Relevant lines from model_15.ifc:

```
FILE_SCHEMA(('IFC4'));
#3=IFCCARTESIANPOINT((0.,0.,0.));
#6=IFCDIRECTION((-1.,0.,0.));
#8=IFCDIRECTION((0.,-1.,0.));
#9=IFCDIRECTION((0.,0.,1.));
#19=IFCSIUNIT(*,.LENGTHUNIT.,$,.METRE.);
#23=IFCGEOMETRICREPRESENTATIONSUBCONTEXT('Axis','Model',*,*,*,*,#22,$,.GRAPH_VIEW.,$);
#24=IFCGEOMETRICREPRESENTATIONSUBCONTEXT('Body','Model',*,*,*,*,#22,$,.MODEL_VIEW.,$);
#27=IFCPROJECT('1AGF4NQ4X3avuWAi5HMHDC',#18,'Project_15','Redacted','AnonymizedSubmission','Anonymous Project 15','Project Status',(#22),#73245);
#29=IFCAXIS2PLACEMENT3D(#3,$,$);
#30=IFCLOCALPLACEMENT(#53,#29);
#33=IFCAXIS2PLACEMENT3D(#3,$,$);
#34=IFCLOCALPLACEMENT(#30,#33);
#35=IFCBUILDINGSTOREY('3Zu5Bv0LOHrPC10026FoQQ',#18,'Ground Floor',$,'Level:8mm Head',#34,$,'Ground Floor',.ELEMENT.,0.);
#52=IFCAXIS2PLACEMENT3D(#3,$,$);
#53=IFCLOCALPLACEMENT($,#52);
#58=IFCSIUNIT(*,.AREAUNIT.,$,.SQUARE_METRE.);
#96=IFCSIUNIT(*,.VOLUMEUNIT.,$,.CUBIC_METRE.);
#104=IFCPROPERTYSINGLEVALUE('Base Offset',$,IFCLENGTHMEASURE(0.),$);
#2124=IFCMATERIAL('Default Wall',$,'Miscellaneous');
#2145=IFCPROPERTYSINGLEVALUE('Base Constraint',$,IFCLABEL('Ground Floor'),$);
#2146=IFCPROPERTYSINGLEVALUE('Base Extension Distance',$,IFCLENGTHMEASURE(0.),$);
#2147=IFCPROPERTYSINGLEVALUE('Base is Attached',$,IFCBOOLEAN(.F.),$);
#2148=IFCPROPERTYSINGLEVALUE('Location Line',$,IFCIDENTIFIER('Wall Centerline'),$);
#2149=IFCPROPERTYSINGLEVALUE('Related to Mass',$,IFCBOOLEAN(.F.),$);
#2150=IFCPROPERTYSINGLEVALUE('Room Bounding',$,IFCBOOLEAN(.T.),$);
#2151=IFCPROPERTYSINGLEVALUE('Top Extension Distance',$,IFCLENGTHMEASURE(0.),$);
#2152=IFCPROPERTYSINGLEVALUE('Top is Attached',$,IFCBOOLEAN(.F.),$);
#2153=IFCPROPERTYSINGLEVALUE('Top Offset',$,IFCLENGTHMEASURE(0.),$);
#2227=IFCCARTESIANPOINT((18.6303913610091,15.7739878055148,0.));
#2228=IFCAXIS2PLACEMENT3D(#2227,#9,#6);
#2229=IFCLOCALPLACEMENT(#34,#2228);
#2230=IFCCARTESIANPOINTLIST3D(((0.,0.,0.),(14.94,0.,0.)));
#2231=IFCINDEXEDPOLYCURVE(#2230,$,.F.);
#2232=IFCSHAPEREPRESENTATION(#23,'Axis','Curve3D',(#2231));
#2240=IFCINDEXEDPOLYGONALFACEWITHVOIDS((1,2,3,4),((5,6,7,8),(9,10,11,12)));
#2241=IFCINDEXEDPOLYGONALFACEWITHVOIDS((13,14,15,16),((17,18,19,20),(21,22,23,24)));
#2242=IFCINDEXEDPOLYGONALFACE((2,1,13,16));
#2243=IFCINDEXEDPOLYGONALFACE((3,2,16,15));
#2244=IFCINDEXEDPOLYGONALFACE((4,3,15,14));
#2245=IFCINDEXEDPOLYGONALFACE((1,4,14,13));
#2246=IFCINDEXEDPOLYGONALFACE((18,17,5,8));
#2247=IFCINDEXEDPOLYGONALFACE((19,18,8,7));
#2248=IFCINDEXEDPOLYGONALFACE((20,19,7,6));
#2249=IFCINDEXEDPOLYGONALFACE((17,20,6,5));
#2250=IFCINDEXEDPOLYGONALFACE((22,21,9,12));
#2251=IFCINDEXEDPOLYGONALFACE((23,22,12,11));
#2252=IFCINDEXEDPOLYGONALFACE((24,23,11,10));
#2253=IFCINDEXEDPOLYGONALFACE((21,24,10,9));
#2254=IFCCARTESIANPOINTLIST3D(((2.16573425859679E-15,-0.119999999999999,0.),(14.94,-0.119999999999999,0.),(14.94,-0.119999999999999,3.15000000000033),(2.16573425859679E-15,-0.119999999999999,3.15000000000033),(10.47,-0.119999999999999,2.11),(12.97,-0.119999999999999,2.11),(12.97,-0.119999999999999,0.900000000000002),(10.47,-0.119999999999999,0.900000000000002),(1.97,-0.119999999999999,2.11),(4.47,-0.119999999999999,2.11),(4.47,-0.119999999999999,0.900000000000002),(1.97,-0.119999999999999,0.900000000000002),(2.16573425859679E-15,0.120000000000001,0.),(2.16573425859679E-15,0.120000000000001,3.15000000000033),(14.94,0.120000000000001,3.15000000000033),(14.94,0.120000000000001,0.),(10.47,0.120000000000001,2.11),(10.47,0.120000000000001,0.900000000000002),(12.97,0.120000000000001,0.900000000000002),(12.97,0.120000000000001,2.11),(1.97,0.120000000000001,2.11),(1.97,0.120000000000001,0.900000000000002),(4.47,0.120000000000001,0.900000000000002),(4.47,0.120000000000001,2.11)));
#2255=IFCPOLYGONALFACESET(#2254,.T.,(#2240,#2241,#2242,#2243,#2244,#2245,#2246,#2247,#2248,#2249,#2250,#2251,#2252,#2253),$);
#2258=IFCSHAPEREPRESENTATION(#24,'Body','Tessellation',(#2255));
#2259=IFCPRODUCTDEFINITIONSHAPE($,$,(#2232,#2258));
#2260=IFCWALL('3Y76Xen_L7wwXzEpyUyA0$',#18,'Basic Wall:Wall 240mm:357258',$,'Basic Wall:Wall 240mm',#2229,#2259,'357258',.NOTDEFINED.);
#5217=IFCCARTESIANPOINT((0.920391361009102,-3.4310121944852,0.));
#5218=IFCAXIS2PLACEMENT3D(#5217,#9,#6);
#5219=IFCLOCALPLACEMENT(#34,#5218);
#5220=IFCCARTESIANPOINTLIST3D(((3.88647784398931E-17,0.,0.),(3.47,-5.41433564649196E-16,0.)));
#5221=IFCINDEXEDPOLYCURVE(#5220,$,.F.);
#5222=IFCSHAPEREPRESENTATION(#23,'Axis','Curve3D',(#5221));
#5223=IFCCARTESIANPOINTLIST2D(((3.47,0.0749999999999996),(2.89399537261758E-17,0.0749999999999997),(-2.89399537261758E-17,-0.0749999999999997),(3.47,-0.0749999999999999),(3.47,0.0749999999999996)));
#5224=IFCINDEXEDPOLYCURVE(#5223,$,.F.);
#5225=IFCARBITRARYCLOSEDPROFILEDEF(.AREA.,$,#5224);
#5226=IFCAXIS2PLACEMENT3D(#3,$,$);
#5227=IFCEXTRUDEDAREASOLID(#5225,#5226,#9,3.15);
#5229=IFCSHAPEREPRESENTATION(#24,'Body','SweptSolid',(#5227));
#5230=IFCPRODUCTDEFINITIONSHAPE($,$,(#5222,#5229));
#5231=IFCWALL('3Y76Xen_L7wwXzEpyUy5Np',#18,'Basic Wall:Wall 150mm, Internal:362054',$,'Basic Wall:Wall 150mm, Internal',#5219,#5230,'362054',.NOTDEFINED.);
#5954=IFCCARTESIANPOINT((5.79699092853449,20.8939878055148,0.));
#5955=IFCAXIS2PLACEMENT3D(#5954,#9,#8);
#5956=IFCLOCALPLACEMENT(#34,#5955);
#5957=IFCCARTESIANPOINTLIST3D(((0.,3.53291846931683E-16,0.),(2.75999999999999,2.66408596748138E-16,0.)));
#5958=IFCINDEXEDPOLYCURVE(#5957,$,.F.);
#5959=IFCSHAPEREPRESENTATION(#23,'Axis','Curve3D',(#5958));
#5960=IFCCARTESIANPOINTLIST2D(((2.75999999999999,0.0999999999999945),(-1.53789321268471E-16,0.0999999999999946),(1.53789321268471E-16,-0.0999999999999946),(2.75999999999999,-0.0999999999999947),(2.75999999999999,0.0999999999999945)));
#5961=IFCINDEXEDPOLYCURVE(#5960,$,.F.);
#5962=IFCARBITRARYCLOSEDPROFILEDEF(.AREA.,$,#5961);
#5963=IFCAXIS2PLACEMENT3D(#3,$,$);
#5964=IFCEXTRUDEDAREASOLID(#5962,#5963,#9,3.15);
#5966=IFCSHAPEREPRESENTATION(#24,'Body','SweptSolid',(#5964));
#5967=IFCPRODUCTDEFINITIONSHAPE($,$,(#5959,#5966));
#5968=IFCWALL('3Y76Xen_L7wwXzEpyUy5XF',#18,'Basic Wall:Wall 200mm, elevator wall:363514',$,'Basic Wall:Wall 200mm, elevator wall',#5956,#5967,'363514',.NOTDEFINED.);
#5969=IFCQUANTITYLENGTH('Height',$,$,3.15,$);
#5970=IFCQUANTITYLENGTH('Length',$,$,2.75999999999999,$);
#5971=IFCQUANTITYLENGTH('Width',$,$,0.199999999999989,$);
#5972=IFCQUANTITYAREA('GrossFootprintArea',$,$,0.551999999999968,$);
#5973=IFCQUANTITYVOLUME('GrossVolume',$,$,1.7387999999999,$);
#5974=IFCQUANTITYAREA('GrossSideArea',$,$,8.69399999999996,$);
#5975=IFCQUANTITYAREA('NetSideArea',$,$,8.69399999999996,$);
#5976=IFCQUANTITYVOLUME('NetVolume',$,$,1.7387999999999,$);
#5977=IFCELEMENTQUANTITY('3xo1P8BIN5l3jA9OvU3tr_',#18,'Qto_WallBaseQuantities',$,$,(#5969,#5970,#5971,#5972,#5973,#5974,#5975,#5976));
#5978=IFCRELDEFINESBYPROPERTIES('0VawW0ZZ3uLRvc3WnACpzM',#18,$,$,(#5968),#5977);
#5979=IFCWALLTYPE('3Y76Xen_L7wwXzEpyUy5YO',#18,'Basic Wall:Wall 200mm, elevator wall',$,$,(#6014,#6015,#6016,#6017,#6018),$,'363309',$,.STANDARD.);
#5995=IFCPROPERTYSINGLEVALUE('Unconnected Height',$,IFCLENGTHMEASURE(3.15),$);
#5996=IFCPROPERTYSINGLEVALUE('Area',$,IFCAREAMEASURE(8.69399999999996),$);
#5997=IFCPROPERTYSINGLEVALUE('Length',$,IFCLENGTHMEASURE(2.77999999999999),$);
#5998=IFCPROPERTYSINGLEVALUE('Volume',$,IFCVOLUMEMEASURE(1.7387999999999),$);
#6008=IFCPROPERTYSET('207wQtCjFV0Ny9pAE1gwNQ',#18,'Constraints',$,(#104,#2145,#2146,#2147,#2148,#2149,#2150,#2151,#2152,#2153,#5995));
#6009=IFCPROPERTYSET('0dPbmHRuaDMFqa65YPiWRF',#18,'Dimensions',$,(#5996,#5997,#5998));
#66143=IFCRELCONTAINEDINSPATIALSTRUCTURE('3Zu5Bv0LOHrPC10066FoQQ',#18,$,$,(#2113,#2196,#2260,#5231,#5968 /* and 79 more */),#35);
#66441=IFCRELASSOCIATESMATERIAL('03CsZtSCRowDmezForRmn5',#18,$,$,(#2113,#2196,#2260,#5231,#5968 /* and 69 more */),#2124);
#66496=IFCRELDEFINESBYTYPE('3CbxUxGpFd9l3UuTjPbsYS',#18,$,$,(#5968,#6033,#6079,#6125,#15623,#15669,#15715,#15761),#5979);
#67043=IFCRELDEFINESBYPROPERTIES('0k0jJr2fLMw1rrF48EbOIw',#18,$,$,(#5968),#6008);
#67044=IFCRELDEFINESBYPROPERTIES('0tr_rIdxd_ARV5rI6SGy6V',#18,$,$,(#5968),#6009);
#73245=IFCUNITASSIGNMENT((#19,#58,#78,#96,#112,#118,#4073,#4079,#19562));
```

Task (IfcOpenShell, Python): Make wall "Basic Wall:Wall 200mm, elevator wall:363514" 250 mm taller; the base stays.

```python
import ifcopenshell
import ifcopenshell.api.pset
import ifcopenshell.geom
import ifcopenshell.util.element
import ifcopenshell.util.representation
import ifcopenshell.util.shape
import ifcopenshell.util.unit

model = ifcopenshell.open("model_15.ifc")
unit_scale = ifcopenshell.util.unit.calculate_unit_scale(model)
area_scale = ifcopenshell.util.unit.calculate_unit_scale(model, "AREAUNIT")
volume_scale = ifcopenshell.util.unit.calculate_unit_scale(model, "VOLUMEUNIT")
settings = ifcopenshell.geom.settings()


def volume(element):
    """Net volume in cubic metres, openings subtracted."""
    shape = ifcopenshell.geom.create_shape(settings, element)
    return ifcopenshell.util.shape.get_volume(shape.geometry)


wall = model.by_guid("3Y76Xen_L7wwXzEpyUy5XF")
before = volume(wall)

body = ifcopenshell.util.representation.get_representation(wall, "Model", "Body")
solid = body.Items[0]
old_height = solid.Depth
solid.Depth += 0.25 / unit_scale
after = volume(wall)
thickness = 0.2  # wall thickness in metres

# Update the stored height, areas and volumes.
qto = model.by_id(ifcopenshell.util.element.get_pset(wall, "Qto_WallBaseQuantities", should_inherit=False)["id"])
ifcopenshell.api.pset.edit_qto(model, qto=qto, properties={
    "Height": solid.Depth,
    "GrossVolume": ifcopenshell.util.element.get_pset(wall, "Qto_WallBaseQuantities", "GrossVolume") * solid.Depth / old_height,
    "GrossSideArea": ifcopenshell.util.element.get_pset(wall, "Qto_WallBaseQuantities", "GrossSideArea") * solid.Depth / old_height,
    "NetSideArea": after / thickness / area_scale,
    "NetVolume": after / volume_scale,
})
pset = model.by_id(ifcopenshell.util.element.get_pset(wall, "Constraints", should_inherit=False)["id"])
ifcopenshell.api.pset.edit_pset(model, pset=pset, properties={
    "Unconnected Height": model.create_entity("IfcLengthMeasure", solid.Depth),
})
pset = model.by_id(ifcopenshell.util.element.get_pset(wall, "Dimensions", should_inherit=False)["id"])
ifcopenshell.api.pset.edit_pset(model, pset=pset, properties={
    "Area": model.create_entity("IfcAreaMeasure", after / thickness / area_scale),
    "Volume": model.create_entity("IfcVolumeMeasure", after / volume_scale),
})

print(f"height {old_height:g} -> {solid.Depth:g}, volume {before:.3f} -> {after:.3f} m3")

model.write("model_15-out.ifc")
```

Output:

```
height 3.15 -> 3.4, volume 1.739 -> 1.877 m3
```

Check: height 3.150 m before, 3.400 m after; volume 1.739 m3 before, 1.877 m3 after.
